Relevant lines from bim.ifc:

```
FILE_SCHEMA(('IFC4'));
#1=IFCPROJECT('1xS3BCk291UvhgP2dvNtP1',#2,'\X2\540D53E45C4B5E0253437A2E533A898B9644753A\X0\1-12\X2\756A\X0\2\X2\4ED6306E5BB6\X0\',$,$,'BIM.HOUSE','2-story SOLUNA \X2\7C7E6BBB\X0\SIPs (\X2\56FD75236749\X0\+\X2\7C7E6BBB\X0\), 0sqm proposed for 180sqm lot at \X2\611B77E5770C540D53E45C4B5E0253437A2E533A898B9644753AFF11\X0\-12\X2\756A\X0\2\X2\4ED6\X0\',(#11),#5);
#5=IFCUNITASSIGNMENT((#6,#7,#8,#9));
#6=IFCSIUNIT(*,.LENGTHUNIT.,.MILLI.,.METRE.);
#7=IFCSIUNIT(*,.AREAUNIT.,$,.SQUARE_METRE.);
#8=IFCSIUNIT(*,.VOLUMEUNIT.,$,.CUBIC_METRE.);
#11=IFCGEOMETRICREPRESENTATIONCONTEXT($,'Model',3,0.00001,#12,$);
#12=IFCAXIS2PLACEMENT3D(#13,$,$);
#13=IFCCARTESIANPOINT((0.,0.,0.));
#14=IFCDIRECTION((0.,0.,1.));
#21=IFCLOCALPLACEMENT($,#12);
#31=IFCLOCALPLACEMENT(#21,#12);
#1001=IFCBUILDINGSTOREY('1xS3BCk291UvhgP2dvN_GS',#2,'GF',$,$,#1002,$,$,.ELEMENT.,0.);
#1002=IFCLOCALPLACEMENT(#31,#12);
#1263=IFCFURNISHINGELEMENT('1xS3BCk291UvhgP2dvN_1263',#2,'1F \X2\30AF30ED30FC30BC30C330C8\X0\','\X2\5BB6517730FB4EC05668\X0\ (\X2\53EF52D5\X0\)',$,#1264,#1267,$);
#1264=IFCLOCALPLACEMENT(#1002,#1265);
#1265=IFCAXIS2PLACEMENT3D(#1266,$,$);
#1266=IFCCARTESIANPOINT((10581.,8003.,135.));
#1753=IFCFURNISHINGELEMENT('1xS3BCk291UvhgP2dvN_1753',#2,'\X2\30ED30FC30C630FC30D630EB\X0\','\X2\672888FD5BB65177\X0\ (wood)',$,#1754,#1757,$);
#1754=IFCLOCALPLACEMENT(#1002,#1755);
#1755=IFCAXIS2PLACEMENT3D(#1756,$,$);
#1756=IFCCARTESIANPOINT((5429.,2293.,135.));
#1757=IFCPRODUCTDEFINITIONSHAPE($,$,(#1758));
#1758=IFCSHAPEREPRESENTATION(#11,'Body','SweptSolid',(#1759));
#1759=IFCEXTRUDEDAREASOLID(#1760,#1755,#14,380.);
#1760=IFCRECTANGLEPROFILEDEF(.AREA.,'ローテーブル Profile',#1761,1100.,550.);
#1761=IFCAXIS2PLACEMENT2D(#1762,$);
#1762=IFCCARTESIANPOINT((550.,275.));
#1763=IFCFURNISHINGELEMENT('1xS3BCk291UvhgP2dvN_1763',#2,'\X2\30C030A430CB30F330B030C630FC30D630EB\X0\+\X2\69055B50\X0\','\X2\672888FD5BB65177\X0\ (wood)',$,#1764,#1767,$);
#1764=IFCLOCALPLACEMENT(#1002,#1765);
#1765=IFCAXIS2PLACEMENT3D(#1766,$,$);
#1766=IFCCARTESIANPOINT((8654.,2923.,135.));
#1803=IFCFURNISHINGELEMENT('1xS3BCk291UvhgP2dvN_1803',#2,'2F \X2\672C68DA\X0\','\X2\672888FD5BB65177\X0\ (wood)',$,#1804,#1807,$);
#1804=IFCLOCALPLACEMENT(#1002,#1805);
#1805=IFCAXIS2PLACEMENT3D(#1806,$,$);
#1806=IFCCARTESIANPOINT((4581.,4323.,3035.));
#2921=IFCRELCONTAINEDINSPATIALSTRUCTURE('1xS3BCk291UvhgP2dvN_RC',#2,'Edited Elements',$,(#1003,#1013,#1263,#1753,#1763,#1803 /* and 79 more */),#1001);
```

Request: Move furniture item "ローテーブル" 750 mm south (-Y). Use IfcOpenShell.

```python
import ifcopenshell
import ifcopenshell.api.geometry
import ifcopenshell.util.placement
import ifcopenshell.util.unit

model = ifcopenshell.open("bim.ifc")
unit_scale = ifcopenshell.util.unit.calculate_unit_scale(model)

item = model.by_guid("1xS3BCk291UvhgP2dvN_1753")
matrix = ifcopenshell.util.placement.get_local_placement(item.ObjectPlacement)
matrix[1, 3] -= 0.75 / unit_scale
ifcopenshell.api.geometry.edit_object_placement(model, product=item, matrix=matrix, is_si=False)

print(ifcopenshell.util.placement.get_local_placement(item.ObjectPlacement).round(3) + 0.0)

model.write("bim_updated.ifc")
```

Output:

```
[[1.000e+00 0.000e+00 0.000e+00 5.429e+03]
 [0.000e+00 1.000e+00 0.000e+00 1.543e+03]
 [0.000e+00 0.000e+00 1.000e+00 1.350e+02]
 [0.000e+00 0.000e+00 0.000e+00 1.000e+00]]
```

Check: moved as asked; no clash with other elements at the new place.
